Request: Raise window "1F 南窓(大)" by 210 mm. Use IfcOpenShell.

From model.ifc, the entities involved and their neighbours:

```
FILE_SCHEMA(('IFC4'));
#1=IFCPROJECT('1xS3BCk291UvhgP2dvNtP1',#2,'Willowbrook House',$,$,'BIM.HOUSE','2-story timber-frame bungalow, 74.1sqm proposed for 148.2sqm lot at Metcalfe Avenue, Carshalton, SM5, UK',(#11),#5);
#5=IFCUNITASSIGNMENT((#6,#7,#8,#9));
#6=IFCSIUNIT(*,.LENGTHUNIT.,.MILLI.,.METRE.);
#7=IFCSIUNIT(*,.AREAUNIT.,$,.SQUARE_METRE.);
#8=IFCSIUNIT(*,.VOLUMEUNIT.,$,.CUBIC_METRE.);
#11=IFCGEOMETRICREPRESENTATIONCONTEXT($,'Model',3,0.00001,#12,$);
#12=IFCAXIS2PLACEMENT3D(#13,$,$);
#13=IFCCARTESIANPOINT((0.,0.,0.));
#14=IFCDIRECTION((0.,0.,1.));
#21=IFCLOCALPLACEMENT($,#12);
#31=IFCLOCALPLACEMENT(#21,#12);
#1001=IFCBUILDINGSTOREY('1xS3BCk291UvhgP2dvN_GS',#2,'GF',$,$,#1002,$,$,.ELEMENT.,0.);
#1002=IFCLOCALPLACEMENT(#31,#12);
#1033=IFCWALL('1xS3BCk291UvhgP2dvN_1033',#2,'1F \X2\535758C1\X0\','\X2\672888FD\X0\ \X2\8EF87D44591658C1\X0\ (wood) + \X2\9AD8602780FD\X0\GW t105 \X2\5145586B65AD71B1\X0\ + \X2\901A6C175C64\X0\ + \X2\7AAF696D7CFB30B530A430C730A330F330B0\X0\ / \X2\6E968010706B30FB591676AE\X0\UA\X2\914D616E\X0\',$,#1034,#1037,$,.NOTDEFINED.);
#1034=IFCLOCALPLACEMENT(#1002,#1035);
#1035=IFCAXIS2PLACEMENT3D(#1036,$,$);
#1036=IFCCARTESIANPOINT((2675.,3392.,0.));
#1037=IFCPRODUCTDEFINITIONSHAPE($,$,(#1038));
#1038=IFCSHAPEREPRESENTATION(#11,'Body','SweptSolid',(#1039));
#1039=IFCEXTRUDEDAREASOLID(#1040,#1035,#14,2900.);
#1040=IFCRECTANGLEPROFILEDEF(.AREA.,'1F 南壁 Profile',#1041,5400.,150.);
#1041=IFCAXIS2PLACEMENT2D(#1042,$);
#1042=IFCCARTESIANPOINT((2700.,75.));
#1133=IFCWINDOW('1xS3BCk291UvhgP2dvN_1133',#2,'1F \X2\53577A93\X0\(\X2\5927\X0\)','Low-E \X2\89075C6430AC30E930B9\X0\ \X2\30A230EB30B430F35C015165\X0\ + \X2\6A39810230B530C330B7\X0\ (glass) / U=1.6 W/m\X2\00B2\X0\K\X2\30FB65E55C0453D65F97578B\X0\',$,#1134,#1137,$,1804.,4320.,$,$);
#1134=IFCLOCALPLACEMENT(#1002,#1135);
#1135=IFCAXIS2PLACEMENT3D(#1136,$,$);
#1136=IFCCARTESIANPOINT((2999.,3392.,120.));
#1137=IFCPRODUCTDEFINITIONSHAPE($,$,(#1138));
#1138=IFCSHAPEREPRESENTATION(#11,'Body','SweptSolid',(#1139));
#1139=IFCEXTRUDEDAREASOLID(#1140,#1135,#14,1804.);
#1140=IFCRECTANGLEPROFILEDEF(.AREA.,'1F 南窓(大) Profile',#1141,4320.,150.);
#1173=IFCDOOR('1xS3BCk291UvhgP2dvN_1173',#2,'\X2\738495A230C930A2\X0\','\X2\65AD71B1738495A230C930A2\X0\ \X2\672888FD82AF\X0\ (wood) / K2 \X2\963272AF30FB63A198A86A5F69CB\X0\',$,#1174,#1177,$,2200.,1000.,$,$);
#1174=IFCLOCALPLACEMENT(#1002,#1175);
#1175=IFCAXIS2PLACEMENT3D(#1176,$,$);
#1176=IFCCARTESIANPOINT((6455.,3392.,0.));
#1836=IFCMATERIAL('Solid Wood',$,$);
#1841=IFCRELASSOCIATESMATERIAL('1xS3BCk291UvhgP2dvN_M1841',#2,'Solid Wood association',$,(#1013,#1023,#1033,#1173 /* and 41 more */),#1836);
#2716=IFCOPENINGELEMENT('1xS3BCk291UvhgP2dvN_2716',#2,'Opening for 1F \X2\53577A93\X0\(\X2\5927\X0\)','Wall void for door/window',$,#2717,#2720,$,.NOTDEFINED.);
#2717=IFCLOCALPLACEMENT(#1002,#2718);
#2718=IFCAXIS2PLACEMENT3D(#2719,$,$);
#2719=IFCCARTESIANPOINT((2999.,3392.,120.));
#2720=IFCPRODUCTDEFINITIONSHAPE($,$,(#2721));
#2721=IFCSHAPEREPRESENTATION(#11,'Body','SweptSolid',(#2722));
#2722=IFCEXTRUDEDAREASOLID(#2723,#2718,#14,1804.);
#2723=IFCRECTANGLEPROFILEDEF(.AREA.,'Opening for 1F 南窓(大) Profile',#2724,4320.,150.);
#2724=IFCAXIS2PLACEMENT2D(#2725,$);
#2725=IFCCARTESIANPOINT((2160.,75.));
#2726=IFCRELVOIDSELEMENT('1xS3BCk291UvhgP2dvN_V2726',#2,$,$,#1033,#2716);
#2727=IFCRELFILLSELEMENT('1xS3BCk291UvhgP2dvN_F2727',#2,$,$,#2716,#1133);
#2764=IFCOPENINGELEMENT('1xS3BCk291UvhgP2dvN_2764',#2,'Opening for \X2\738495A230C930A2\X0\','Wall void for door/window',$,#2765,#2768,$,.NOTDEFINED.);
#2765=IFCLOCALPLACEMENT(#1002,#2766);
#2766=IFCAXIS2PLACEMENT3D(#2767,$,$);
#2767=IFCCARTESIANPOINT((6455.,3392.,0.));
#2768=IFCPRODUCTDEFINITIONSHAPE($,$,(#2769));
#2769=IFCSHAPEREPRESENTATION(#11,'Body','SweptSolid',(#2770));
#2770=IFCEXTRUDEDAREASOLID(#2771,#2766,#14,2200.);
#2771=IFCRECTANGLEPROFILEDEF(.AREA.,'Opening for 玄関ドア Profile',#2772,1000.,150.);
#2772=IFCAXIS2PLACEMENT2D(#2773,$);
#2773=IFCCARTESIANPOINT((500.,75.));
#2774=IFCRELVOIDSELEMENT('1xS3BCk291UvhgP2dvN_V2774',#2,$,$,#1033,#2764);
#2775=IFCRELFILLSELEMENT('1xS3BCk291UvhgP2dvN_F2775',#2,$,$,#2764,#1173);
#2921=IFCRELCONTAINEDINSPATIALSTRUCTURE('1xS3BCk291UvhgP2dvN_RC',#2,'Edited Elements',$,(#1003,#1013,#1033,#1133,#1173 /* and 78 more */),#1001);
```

```python
import numpy as np
import ifcopenshell
import ifcopenshell.api.geometry
import ifcopenshell.util.placement
import ifcopenshell.util.unit

model = ifcopenshell.open("model.ifc")
unit_scale = ifcopenshell.util.unit.calculate_unit_scale(model)

window = model.by_guid("1xS3BCk291UvhgP2dvN_1133")
opening = window.FillsVoids[0].RelatingOpeningElement
dz = 210.0

shift = np.array([0.0, 0.0, dz])
# The window is not placed relative to its opening, so move both.
for product in (opening, window):
    matrix = ifcopenshell.util.placement.get_local_placement(product.ObjectPlacement)
    matrix[:3, 3] += shift
    ifcopenshell.api.geometry.edit_object_placement(model, product=product, matrix=matrix, is_si=False)

print(f"moved by {dz * unit_scale:+.3f} m")

model.write("model_v2.ifc")
```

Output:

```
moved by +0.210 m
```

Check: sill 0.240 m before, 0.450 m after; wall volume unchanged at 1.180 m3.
